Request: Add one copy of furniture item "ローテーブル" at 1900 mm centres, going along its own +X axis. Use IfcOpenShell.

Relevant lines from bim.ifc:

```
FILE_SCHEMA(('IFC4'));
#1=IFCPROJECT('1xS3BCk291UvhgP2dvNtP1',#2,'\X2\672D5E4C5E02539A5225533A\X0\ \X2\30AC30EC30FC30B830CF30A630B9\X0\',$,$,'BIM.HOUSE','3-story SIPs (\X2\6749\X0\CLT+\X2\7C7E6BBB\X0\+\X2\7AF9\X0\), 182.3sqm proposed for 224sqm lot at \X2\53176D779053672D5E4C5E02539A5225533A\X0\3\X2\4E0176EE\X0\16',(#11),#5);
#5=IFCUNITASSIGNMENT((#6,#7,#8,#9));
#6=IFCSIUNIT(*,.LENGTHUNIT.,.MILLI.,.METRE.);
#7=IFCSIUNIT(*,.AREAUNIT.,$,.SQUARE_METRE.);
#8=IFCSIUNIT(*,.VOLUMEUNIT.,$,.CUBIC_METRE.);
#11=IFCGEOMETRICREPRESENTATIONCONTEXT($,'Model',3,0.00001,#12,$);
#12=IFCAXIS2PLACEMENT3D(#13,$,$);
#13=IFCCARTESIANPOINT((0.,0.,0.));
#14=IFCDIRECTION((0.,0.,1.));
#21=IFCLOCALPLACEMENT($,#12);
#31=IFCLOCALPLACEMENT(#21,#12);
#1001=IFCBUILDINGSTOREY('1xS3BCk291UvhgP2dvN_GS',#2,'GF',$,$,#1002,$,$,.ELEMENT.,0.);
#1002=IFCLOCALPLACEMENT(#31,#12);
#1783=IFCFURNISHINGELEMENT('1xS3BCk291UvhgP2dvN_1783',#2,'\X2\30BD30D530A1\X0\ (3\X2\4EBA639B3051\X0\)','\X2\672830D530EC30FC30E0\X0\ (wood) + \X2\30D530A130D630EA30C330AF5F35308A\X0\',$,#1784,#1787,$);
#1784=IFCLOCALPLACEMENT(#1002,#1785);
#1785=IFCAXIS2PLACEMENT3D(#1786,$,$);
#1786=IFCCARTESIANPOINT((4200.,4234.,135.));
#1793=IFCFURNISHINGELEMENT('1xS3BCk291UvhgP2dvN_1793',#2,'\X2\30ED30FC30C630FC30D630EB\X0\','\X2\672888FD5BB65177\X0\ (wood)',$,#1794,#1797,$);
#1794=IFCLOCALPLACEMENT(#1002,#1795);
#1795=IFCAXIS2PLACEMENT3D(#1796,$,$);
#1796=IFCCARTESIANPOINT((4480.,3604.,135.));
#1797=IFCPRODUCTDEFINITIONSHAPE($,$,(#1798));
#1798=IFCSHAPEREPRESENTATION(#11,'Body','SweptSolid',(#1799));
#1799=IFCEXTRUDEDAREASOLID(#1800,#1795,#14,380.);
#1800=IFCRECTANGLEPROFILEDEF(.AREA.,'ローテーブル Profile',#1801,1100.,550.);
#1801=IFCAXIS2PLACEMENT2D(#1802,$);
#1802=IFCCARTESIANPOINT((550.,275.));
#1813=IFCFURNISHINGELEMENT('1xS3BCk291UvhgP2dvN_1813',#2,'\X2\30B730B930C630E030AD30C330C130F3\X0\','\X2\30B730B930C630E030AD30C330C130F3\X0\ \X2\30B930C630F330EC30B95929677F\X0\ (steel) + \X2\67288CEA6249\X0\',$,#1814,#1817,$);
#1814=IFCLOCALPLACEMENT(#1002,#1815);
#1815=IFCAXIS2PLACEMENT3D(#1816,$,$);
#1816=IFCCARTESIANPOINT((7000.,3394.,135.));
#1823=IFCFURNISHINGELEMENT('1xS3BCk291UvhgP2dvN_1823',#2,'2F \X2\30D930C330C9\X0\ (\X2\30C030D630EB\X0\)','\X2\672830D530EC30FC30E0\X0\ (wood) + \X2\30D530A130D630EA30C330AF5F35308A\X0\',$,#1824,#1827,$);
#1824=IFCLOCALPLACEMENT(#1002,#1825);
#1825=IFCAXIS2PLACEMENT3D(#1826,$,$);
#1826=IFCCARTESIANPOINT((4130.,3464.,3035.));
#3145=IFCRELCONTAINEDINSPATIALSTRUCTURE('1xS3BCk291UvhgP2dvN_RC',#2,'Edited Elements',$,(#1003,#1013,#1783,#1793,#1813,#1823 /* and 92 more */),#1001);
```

```python
import ifcopenshell
import ifcopenshell.api.geometry
import ifcopenshell.api.root
import ifcopenshell.util.element
import ifcopenshell.util.placement
import ifcopenshell.util.unit

model = ifcopenshell.open("bim.ifc")
unit_scale = ifcopenshell.util.unit.calculate_unit_scale(model)


def reuse_history(source, copy):
    """copy_class also copies each property set's owner history, people and application; keep the originals."""
    for rel in copy.IsDefinedBy:
        if rel.is_a("IfcRelDefinesByProperties") and (history := rel.RelatingPropertyDefinition.OwnerHistory):
            rel.RelatingPropertyDefinition.OwnerHistory = source.OwnerHistory
            ifcopenshell.util.element.remove_deep2(model, history)


source = model.by_guid("1xS3BCk291UvhgP2dvN_1793")
base = ifcopenshell.util.placement.get_local_placement(source.ObjectPlacement)
step = base[:3, 0] * 1.9 / unit_scale

for i in range(1, 2):
    copy = ifcopenshell.api.root.copy_class(model, product=source)
    copy.Representation = ifcopenshell.util.element.copy_deep(
        model, source.Representation, exclude=["IfcGeometricRepresentationContext", "IfcRepresentationMap"]
    )
    reuse_history(source, copy)
    matrix = base.copy()
    matrix[:3, 3] += i * step
    print("added at", matrix[:3, 3].round(3) + 0.0)
    ifcopenshell.api.geometry.edit_object_placement(model, product=copy, matrix=matrix, is_si=False)

model.write("bim_v2.ifc")
```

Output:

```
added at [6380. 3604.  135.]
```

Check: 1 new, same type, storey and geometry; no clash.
